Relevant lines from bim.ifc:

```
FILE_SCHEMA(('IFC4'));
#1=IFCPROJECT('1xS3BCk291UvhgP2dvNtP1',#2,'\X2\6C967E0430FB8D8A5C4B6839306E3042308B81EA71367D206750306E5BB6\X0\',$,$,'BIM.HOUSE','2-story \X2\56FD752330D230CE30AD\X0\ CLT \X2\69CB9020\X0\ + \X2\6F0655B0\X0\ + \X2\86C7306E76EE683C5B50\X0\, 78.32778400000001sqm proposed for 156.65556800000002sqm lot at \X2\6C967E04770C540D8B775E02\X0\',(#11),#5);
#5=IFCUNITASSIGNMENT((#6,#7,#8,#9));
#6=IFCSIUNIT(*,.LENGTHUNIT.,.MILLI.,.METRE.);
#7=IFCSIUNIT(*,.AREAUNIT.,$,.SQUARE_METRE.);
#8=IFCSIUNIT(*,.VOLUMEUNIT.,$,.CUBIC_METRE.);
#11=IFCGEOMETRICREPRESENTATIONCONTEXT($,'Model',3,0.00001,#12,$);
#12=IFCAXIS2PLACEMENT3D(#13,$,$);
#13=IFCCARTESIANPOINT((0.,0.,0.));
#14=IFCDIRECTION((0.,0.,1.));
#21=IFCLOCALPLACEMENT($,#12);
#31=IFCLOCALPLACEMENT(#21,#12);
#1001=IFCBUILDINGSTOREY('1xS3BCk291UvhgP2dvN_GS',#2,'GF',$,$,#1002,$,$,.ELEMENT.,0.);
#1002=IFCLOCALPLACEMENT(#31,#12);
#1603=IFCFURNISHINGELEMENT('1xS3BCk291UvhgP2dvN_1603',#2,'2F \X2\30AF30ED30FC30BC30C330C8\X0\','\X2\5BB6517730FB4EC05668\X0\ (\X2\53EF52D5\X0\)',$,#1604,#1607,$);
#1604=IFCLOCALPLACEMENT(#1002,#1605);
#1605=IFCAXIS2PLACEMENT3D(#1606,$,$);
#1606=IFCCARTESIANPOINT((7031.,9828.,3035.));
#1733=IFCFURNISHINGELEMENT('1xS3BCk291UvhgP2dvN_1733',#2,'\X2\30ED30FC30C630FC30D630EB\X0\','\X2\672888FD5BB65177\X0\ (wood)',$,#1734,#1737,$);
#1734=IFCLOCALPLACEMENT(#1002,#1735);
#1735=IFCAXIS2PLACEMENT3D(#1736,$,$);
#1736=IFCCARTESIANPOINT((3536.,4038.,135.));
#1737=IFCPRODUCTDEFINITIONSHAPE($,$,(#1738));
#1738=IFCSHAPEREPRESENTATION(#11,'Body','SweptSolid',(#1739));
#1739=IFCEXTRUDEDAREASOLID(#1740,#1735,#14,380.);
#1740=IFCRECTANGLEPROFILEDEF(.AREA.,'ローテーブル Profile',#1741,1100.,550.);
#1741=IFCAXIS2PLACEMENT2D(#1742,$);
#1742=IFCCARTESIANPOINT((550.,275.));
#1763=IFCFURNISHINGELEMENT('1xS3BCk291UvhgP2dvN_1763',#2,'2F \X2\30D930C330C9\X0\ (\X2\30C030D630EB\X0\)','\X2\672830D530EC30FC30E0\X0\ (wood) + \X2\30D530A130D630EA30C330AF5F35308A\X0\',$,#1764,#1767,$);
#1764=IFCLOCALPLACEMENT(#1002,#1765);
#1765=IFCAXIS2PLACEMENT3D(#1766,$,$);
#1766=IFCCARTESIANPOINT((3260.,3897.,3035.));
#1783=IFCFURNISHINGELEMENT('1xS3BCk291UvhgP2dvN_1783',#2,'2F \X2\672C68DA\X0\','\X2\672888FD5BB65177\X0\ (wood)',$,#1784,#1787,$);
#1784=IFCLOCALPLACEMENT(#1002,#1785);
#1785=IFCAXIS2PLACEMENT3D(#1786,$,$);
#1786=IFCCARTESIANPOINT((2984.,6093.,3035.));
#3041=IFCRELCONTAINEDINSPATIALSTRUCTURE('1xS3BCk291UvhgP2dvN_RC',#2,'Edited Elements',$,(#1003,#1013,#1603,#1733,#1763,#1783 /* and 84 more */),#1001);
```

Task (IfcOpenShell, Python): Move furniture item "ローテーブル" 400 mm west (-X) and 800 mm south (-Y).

```python
import ifcopenshell
import ifcopenshell.api.geometry
import ifcopenshell.util.placement
import ifcopenshell.util.unit

model = ifcopenshell.open("bim.ifc")
unit_scale = ifcopenshell.util.unit.calculate_unit_scale(model)

item = model.by_id(1733)
matrix = ifcopenshell.util.placement.get_local_placement(item.ObjectPlacement)
matrix[0, 3] -= 0.4 / unit_scale
matrix[1, 3] -= 0.8 / unit_scale
ifcopenshell.api.geometry.edit_object_placement(model, product=item, matrix=matrix, is_si=False)

print(ifcopenshell.util.placement.get_local_placement(item.ObjectPlacement).round(3) + 0.0)

model.write("bim_edited.ifc")
```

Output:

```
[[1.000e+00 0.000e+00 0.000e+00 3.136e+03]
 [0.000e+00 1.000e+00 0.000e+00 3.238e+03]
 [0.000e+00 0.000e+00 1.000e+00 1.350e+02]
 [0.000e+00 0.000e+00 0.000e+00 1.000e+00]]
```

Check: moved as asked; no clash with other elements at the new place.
